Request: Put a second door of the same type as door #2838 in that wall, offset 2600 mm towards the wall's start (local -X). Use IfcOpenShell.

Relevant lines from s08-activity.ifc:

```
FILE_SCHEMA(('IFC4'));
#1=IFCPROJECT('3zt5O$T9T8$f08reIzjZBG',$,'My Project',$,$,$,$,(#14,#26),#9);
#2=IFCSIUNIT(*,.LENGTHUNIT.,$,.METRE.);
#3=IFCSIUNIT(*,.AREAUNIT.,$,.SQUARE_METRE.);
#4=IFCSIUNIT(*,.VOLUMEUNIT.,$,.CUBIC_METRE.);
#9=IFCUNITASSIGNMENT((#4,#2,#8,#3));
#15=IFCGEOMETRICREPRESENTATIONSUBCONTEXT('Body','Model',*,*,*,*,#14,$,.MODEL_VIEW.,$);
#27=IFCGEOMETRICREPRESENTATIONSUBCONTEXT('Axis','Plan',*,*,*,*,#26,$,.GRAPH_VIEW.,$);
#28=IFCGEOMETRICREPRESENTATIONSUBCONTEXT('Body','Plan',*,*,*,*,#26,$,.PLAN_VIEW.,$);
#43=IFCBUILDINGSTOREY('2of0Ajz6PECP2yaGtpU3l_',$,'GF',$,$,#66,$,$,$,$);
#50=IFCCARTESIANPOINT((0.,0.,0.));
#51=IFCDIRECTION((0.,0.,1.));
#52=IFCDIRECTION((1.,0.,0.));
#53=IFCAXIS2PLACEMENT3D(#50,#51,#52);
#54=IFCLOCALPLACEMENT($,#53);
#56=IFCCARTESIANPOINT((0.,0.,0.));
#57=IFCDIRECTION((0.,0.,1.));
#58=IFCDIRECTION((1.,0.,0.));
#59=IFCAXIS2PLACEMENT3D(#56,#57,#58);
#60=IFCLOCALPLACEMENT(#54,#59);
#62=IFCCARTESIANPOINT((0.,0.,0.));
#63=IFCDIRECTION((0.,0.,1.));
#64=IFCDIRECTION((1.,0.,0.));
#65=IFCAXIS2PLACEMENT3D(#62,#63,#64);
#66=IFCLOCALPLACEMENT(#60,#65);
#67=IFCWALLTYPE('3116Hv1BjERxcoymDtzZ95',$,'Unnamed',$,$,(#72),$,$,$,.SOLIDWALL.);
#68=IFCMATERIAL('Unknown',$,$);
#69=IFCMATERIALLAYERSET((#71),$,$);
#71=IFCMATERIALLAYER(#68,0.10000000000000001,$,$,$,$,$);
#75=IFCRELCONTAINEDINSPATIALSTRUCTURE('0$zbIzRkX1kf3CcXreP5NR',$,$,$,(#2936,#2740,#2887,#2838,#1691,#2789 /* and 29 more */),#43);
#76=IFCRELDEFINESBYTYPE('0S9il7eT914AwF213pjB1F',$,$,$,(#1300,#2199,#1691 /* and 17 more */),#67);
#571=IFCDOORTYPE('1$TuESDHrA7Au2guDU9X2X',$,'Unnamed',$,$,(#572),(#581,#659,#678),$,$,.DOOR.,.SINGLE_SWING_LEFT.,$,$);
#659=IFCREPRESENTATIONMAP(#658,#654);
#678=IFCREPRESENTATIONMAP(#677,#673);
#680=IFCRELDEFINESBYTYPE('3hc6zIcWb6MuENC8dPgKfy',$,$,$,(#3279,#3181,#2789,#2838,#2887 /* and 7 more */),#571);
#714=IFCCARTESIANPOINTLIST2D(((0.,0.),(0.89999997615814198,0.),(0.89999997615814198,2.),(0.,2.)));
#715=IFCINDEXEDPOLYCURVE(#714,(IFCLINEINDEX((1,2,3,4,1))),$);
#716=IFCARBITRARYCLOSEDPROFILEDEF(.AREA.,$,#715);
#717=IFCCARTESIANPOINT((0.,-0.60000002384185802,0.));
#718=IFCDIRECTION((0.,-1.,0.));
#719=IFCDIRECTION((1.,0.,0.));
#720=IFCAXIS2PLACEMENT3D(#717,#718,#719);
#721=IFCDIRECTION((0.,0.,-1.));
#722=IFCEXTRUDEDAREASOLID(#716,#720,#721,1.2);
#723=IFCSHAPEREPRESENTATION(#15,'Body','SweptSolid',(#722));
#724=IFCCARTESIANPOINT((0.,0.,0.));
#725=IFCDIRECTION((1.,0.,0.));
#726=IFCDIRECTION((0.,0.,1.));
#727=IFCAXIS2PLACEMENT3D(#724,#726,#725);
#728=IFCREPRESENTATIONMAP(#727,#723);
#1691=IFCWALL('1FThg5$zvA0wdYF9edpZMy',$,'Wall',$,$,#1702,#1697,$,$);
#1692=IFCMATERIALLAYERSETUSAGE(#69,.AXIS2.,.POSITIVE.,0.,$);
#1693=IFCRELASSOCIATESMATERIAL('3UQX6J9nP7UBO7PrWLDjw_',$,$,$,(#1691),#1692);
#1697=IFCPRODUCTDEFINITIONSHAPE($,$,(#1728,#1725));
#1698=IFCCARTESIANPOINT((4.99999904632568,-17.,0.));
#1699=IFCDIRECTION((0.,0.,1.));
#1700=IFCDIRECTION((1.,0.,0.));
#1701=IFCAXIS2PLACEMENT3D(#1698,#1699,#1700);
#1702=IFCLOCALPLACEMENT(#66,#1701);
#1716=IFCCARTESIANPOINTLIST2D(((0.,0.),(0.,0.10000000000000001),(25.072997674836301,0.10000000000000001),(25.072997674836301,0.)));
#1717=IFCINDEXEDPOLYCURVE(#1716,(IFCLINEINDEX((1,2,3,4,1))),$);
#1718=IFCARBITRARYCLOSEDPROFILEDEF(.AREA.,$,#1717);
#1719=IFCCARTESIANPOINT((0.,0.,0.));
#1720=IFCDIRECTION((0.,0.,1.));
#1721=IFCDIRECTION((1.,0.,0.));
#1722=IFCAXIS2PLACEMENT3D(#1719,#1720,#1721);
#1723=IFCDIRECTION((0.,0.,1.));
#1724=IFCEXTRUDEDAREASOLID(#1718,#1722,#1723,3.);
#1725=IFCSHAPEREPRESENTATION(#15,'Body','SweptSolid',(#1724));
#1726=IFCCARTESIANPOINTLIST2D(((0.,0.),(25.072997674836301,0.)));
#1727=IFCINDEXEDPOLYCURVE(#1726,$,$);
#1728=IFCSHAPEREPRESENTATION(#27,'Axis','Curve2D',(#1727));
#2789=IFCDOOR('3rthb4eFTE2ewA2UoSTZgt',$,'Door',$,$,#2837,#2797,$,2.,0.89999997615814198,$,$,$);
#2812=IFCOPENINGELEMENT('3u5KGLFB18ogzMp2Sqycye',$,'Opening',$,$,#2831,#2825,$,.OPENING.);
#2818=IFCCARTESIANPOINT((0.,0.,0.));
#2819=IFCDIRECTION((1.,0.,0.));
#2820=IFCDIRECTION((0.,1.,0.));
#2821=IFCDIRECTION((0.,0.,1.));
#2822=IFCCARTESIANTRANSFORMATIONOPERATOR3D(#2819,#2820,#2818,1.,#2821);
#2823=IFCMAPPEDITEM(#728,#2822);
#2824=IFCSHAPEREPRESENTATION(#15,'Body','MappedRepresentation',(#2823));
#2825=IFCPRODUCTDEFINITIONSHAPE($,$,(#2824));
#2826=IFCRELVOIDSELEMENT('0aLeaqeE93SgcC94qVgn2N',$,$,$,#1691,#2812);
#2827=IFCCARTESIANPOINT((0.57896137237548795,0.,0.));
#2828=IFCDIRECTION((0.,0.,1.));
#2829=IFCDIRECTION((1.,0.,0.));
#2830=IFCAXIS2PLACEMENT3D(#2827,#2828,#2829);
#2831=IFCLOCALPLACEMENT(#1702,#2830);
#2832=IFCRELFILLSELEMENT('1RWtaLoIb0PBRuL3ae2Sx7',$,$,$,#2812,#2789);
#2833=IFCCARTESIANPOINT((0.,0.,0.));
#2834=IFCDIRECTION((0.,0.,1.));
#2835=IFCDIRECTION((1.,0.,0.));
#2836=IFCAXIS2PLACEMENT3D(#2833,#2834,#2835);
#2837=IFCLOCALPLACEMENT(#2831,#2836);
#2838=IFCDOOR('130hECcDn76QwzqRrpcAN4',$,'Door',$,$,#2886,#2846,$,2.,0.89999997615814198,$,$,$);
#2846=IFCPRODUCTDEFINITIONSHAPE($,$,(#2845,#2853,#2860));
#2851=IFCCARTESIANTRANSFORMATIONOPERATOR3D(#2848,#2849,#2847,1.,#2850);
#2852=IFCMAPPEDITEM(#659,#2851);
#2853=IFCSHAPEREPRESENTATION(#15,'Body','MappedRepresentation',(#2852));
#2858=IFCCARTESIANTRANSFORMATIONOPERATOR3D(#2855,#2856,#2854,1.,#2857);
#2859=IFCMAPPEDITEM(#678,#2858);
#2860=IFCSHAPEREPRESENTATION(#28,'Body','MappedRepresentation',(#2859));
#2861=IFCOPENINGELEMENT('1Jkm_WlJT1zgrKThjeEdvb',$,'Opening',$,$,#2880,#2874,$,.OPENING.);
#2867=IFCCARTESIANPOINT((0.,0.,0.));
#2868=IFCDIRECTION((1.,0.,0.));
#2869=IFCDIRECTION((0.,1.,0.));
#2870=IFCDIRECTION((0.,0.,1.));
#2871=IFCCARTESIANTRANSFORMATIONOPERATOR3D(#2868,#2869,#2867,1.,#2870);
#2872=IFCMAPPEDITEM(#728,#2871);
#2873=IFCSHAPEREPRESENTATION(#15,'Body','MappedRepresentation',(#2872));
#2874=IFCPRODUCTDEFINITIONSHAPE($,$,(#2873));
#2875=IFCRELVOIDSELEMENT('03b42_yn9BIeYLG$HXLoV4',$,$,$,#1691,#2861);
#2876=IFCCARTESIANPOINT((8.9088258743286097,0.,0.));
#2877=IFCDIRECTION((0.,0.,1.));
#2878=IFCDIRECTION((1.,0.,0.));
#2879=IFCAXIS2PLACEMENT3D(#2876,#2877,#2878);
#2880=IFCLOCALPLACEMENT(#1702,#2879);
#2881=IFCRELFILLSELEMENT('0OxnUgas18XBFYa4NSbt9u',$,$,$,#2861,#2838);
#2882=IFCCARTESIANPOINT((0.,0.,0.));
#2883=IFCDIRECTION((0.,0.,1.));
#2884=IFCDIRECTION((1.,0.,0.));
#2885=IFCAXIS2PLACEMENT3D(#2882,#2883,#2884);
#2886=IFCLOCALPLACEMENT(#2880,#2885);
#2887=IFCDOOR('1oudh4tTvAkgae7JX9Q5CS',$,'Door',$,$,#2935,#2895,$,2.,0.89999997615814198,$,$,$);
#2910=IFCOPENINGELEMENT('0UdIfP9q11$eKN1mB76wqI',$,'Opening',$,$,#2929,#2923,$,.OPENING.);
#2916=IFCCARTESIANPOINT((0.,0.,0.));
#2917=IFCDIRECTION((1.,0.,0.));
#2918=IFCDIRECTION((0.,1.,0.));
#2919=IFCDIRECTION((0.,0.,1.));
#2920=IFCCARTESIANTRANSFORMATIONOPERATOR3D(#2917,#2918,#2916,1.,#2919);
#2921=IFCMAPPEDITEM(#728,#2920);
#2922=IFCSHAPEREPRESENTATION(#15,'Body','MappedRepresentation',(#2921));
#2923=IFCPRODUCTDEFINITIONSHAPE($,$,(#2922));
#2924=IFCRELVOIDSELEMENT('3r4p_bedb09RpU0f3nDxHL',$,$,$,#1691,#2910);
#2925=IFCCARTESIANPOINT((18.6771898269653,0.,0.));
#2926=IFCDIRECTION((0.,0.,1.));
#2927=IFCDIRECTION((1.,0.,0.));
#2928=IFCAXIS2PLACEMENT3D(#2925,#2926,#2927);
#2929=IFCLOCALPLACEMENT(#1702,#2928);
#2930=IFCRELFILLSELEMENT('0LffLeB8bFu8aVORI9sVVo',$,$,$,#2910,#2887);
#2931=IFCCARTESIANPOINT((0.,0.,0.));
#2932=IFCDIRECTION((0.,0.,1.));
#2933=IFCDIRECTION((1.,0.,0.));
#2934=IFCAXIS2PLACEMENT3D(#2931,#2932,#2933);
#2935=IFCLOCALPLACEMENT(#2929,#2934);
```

```python
import ifcopenshell
import ifcopenshell.api.feature
import ifcopenshell.api.geometry
import ifcopenshell.api.root
import ifcopenshell.geom
import ifcopenshell.util.element
import ifcopenshell.util.placement
import ifcopenshell.util.shape

model = ifcopenshell.open("s08-activity.ifc")
settings = ifcopenshell.geom.settings()


def volume(element):
    """Net volume in cubic metres, openings subtracted."""
    shape = ifcopenshell.geom.create_shape(settings, element)
    return ifcopenshell.util.shape.get_volume(shape.geometry)


door = model.by_guid("130hECcDn76QwzqRrpcAN4")
opening = door.FillsVoids[0].RelatingOpeningElement
wall = opening.VoidsElements[0].RelatingBuildingElement
before = volume(wall)
shift = ifcopenshell.util.placement.get_local_placement(wall.ObjectPlacement)[:3, 0] * -2.6

# copy_class copies the void relationship, type, container and properties, but no geometry.
new_opening = ifcopenshell.api.root.copy_class(model, product=opening)
new_opening.Representation = ifcopenshell.util.element.copy_deep(
    model, opening.Representation, exclude=["IfcGeometricRepresentationContext", "IfcRepresentationMap"]
)
new_door = ifcopenshell.api.root.copy_class(model, product=door)
new_door.Representation = ifcopenshell.util.element.copy_deep(
    model, door.Representation, exclude=["IfcGeometricRepresentationContext", "IfcRepresentationMap"]
)
ifcopenshell.api.feature.add_filling(model, opening=new_opening, element=new_door)

for old, new in ((opening, new_opening), (door, new_door)):
    matrix = ifcopenshell.util.placement.get_local_placement(old.ObjectPlacement)
    matrix[:3, 3] += shift
    ifcopenshell.api.geometry.edit_object_placement(model, product=new, matrix=matrix, is_si=False)

after = volume(wall)

print(f"wall volume {before:.3f} -> {after:.3f} m3")

model.write("s08-activity_edited.ifc")
```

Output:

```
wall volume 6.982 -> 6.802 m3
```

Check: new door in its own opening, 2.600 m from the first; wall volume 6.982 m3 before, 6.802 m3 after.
